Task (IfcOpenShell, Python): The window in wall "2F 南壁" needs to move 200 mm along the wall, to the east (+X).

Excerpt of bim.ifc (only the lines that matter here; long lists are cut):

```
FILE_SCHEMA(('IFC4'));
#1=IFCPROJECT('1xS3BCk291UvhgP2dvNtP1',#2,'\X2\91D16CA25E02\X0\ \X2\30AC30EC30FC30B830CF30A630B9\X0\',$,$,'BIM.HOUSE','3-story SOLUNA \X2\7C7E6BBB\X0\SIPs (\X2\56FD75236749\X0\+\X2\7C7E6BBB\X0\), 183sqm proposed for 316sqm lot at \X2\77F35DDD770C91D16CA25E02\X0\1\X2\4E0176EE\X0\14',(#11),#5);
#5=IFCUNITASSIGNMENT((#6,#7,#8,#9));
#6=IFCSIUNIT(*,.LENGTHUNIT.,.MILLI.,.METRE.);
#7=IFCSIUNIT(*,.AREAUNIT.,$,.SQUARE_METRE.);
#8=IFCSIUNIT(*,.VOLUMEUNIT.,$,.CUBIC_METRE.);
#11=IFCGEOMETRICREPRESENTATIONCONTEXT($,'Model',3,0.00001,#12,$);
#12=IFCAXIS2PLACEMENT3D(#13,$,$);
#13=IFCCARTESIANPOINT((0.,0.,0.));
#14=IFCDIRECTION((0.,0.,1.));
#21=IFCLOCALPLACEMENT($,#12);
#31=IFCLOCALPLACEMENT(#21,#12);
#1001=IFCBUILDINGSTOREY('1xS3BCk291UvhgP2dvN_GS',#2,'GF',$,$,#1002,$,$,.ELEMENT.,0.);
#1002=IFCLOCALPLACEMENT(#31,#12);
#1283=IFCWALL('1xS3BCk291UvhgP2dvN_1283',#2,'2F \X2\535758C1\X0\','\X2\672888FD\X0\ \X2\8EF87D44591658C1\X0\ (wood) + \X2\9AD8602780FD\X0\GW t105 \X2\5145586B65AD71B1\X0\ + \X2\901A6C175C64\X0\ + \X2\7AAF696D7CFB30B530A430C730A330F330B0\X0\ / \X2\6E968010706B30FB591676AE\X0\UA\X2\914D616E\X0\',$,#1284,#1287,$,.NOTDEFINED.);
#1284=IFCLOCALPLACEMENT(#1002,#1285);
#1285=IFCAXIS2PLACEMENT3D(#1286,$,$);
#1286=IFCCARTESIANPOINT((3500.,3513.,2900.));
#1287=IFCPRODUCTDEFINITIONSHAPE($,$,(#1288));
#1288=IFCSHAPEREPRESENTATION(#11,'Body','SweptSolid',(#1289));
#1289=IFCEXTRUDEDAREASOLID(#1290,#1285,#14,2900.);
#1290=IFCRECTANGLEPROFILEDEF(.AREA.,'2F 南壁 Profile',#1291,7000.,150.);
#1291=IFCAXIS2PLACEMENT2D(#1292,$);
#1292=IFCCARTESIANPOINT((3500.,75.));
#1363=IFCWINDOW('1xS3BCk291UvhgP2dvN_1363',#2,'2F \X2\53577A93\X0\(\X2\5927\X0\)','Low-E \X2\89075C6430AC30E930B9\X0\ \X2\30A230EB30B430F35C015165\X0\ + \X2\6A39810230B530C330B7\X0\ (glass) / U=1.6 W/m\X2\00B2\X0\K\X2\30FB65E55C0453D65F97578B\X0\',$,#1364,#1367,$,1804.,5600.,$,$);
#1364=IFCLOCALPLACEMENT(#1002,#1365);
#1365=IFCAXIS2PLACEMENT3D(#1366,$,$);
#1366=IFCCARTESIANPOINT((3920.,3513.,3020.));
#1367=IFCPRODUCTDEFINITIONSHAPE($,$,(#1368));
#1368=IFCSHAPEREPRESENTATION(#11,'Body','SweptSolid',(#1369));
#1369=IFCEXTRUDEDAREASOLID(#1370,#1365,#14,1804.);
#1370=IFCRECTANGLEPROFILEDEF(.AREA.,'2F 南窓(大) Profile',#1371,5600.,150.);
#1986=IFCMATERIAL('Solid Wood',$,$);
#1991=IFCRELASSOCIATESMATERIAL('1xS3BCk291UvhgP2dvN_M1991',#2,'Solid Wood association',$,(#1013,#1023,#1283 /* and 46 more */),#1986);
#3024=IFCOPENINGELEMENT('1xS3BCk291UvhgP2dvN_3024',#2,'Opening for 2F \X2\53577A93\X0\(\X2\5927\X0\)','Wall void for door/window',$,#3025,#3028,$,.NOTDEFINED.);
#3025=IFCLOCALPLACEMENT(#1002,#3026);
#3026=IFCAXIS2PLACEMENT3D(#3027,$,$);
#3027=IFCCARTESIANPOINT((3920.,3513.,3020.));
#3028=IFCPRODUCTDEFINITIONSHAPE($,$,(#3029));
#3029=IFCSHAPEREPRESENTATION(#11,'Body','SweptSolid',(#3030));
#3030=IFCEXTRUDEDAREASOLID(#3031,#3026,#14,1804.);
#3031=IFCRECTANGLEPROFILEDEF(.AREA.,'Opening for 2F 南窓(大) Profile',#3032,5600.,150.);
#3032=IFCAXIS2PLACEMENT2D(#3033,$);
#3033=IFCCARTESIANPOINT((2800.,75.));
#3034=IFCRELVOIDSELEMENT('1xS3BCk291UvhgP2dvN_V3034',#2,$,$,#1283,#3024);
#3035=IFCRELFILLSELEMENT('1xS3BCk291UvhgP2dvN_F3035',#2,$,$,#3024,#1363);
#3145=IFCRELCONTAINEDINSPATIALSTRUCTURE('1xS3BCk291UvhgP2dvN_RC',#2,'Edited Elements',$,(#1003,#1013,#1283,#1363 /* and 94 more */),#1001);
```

```python
import ifcopenshell
import ifcopenshell.api.geometry
import ifcopenshell.util.placement
import ifcopenshell.util.unit

model = ifcopenshell.open("bim.ifc")
unit_scale = ifcopenshell.util.unit.calculate_unit_scale(model)

window = model.by_id(1363)
opening = window.FillsVoids[0].RelatingOpeningElement
wall = opening.VoidsElements[0].RelatingBuildingElement

wall_matrix = ifcopenshell.util.placement.get_local_placement(wall.ObjectPlacement)
shift = wall_matrix[:3, 0] * 0.2 / unit_scale
before = ifcopenshell.util.placement.get_local_placement(window.ObjectPlacement)[:3, 3].copy()

# The window is not placed relative to its opening, so move both.
for product in (opening, window):
    matrix = ifcopenshell.util.placement.get_local_placement(product.ObjectPlacement)
    matrix[:3, 3] += shift
    ifcopenshell.api.geometry.edit_object_placement(model, product=product, matrix=matrix, is_si=False)

after = ifcopenshell.util.placement.get_local_placement(window.ObjectPlacement)[:3, 3]
print("window moved by", (after - before).round(3) + 0.0)

model.write("bim_updated.ifc")
```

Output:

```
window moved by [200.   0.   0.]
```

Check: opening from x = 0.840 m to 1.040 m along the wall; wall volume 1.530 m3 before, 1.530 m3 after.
